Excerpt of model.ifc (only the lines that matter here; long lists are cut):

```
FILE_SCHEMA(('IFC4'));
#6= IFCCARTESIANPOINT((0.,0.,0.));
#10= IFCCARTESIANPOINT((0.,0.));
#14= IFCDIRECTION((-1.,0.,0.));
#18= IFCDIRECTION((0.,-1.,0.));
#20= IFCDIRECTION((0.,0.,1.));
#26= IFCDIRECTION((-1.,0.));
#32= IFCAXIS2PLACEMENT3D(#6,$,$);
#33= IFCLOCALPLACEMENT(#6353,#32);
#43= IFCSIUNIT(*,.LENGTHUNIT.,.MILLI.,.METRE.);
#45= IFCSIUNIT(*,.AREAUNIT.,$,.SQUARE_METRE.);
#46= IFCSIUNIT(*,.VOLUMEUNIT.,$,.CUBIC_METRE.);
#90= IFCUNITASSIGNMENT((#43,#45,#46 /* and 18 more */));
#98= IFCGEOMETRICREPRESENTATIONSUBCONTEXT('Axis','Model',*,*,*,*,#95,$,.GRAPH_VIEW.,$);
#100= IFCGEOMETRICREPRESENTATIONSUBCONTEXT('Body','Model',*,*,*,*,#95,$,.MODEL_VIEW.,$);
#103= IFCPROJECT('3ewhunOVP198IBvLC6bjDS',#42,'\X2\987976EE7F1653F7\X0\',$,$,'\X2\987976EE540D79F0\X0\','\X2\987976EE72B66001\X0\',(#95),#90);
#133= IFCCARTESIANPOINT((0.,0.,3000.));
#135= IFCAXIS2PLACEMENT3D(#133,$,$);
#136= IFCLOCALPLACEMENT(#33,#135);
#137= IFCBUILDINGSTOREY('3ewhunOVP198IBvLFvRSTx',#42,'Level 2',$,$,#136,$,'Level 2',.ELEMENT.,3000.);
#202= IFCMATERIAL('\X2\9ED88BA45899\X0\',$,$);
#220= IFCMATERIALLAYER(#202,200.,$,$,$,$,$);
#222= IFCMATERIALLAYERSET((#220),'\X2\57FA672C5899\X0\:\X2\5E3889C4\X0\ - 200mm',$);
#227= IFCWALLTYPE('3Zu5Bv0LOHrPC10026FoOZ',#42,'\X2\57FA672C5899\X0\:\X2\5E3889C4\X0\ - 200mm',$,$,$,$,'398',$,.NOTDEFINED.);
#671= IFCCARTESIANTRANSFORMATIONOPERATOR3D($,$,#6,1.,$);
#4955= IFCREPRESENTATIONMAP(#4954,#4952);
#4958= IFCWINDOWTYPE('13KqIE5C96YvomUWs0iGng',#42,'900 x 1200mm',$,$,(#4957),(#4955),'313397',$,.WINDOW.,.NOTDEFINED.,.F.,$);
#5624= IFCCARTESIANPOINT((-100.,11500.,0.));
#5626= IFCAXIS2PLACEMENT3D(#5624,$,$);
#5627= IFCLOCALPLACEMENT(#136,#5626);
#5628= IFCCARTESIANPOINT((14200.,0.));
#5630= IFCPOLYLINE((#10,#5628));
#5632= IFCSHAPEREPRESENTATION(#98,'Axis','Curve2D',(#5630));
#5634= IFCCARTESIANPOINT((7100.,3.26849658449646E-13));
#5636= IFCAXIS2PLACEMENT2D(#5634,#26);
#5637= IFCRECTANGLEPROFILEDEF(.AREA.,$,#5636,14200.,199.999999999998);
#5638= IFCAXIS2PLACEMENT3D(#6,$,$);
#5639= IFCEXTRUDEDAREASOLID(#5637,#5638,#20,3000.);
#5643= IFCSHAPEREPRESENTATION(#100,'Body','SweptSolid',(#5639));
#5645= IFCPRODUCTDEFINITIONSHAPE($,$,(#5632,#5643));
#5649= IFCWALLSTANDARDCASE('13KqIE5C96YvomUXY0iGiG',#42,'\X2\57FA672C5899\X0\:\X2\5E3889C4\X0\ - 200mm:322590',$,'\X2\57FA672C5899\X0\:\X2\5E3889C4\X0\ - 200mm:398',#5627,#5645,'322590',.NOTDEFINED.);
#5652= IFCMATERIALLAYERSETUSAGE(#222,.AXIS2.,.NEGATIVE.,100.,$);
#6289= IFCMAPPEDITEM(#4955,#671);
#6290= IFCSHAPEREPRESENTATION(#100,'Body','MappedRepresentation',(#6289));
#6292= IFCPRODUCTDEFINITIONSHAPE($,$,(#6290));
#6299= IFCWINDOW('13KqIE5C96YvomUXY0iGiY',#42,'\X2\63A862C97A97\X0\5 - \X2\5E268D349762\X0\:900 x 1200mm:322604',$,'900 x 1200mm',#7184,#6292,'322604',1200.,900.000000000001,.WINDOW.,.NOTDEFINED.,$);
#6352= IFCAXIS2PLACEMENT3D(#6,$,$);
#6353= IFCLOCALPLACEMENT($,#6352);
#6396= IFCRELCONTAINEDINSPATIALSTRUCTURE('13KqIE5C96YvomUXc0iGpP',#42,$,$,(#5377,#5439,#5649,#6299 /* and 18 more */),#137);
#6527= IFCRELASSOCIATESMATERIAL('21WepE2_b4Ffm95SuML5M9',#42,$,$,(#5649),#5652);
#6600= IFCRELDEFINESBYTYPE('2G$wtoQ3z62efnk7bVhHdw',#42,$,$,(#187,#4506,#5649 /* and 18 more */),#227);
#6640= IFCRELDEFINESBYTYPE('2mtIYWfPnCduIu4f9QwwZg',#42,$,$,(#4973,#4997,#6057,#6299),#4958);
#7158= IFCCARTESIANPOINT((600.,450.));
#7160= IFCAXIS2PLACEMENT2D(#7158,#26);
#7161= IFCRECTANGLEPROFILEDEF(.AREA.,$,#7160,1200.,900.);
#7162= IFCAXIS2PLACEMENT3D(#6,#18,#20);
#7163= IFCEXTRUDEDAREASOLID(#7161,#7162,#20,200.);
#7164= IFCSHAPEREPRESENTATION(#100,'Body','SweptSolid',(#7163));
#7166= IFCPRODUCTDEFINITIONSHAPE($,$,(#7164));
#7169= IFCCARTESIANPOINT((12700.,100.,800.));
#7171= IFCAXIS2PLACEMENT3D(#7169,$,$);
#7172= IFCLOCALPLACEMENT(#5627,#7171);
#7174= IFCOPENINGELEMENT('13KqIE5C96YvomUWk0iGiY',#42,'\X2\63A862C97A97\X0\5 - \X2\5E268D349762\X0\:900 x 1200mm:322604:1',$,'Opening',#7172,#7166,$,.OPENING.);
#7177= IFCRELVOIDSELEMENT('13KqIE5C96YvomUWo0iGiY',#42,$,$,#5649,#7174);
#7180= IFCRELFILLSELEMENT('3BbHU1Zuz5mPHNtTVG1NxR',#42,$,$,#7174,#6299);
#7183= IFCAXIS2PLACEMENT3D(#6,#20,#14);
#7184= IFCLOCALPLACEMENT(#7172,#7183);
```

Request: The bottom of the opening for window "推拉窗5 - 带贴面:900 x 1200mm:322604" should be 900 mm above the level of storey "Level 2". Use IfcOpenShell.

```python
import numpy as np
import ifcopenshell
import ifcopenshell.api.geometry
import ifcopenshell.geom
import ifcopenshell.util.element
import ifcopenshell.util.placement
import ifcopenshell.util.shape
import ifcopenshell.util.unit

model = ifcopenshell.open("model.ifc")
unit_scale = ifcopenshell.util.unit.calculate_unit_scale(model)

window = model.by_id(6299)
opening = window.FillsVoids[0].RelatingOpeningElement
storey = ifcopenshell.util.element.get_container(window, ifc_class="IfcBuildingStorey")
level = ifcopenshell.util.placement.get_local_placement(storey.ObjectPlacement)[2, 3]

# The opening's origin need not be at the sill, so measure its lowest point.
shape = ifcopenshell.geom.create_shape(ifcopenshell.geom.settings(), opening)
bottom = ifcopenshell.util.shape.get_shape_bottom_elevation(shape, shape.geometry) / unit_scale
dz = level + 0.9 / unit_scale - bottom

shift = np.array([0.0, 0.0, dz])
# The window is placed relative to its opening, so it follows when the opening moves.
matrix = ifcopenshell.util.placement.get_local_placement(opening.ObjectPlacement)
matrix[:3, 3] += shift
ifcopenshell.api.geometry.edit_object_placement(
    model, product=opening, matrix=matrix, is_si=False, should_transform_children=True
)

print(f"moved by {dz * unit_scale:+.3f} m")

model.write("model_v2.ifc")
```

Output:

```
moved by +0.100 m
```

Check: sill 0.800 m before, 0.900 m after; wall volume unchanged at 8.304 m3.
